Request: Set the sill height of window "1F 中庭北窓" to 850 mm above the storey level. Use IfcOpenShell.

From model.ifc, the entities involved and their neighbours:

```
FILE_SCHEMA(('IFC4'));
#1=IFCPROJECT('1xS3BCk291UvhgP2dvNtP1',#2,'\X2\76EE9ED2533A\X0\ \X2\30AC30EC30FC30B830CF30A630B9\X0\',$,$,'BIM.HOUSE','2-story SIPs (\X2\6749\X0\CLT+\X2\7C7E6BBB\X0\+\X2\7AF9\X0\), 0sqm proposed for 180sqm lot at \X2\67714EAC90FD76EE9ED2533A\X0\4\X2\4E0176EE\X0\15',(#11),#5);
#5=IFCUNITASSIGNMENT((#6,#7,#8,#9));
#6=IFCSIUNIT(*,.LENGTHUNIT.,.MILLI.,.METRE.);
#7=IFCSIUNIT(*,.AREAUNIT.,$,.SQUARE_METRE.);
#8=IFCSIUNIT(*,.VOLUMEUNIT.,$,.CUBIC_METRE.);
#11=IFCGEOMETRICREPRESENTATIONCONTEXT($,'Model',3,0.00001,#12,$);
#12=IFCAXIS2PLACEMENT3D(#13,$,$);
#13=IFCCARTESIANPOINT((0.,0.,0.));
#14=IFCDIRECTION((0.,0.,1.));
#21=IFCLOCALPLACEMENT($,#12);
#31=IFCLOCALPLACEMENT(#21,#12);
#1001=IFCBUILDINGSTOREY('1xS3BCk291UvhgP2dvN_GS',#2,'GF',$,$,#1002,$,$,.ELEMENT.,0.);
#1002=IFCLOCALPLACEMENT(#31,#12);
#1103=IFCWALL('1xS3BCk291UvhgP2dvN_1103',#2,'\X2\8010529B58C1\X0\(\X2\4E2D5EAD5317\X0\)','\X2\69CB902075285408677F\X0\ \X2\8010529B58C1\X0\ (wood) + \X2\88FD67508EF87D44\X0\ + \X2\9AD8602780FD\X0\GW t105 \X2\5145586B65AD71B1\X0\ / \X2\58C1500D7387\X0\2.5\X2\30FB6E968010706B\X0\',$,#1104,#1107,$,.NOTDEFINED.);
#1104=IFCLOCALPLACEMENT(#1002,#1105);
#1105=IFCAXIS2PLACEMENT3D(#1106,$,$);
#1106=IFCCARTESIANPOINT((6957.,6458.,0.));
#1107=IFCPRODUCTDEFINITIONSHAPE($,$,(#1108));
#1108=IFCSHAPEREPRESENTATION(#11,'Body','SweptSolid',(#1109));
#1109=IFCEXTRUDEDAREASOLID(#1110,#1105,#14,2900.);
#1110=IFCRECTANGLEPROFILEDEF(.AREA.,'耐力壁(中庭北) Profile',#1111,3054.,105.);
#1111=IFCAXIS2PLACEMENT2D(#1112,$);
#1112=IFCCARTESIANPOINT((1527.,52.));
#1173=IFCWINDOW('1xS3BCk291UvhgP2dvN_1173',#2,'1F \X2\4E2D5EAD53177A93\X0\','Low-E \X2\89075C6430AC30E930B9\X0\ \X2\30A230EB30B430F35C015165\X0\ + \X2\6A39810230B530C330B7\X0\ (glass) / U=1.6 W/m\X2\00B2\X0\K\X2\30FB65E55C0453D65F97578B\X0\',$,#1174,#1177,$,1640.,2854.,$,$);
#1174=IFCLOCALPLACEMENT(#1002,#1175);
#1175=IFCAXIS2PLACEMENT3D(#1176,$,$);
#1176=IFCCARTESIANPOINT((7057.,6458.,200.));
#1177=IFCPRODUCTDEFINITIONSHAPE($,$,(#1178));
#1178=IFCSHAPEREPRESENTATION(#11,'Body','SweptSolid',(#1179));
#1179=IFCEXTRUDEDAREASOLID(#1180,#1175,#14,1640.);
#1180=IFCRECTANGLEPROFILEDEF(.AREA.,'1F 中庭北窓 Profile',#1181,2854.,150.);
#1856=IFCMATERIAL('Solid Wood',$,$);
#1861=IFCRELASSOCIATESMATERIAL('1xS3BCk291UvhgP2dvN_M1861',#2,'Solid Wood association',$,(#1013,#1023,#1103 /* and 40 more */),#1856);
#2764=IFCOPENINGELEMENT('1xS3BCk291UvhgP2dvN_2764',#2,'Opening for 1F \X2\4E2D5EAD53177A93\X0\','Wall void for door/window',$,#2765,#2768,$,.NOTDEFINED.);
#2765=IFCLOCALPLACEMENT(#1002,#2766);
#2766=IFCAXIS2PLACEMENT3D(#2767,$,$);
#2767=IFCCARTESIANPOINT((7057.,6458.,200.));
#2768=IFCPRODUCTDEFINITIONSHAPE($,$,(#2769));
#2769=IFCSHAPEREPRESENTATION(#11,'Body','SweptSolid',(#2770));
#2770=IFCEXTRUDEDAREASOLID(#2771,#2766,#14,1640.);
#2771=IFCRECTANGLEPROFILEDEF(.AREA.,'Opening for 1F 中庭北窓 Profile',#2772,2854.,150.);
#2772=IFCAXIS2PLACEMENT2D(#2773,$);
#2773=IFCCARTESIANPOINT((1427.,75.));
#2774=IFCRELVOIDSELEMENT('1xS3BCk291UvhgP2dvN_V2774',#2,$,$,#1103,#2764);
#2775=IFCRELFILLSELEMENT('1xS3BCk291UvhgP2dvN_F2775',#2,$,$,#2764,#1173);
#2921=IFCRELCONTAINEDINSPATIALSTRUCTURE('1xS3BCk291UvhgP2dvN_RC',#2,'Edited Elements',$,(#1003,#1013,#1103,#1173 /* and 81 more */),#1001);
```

```python
import numpy as np
import ifcopenshell
import ifcopenshell.api.geometry
import ifcopenshell.geom
import ifcopenshell.util.element
import ifcopenshell.util.placement
import ifcopenshell.util.shape
import ifcopenshell.util.unit

model = ifcopenshell.open("model.ifc")
unit_scale = ifcopenshell.util.unit.calculate_unit_scale(model)

window = model.by_guid("1xS3BCk291UvhgP2dvN_1173")
opening = window.FillsVoids[0].RelatingOpeningElement
storey = ifcopenshell.util.element.get_container(window, ifc_class="IfcBuildingStorey")
level = ifcopenshell.util.placement.get_local_placement(storey.ObjectPlacement)[2, 3]

# The opening's origin need not be at the sill, so measure its lowest point.
shape = ifcopenshell.geom.create_shape(ifcopenshell.geom.settings(), opening)
bottom = ifcopenshell.util.shape.get_shape_bottom_elevation(shape, shape.geometry) / unit_scale
dz = level + 850.0 - bottom

shift = np.array([0.0, 0.0, dz])
# The window is not placed relative to its opening, so move both.
for product in (opening, window):
    matrix = ifcopenshell.util.placement.get_local_placement(product.ObjectPlacement)
    matrix[:3, 3] += shift
    ifcopenshell.api.geometry.edit_object_placement(model, product=product, matrix=matrix, is_si=False)

print(f"moved by {dz * unit_scale:+.3f} m")

model.write("model_rev.ifc")
```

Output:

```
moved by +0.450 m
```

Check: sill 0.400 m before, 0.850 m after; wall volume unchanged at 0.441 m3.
